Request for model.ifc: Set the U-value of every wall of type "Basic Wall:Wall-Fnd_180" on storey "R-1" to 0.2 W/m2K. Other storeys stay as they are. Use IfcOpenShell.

First a look at what the model holds.

```python
import ifcopenshell
import ifcopenshell.util.element

model = ifcopenshell.open("model.ifc")
print(model.schema)
storey = next(s for s in model.by_type("IfcBuildingStorey") if s.Name == "R-1")
walls = [e for e in ifcopenshell.util.element.get_decomposition(storey) if e.is_a("IfcWall")]
seen = {}
for e in walls:
    element_type = ifcopenshell.util.element.get_type(e)
    key = (element_type.Name if element_type != e and element_type else None, ifcopenshell.util.element.get_pset(e, "Pset_WallCommon", "ThermalTransmittance"))
    seen[key] = seen.get(key, 0) + 1
for (name, value), count in sorted(seen.items(), key=str):
    print(count, "x", name, "|", value)
```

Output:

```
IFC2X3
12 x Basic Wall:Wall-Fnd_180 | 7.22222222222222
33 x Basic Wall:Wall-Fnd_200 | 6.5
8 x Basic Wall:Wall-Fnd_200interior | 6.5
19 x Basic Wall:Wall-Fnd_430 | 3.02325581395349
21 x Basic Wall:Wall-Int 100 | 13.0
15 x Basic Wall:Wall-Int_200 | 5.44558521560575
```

```python
import ifcopenshell
import ifcopenshell.api.pset
import ifcopenshell.util.element

model = ifcopenshell.open("model.ifc")

storey = next(s for s in model.by_type("IfcBuildingStorey") if s.Name == "R-1")
walls = [e for e in ifcopenshell.util.element.get_decomposition(storey) if e.is_a("IfcWall")]

count = 0
for e in walls:
    element_type = ifcopenshell.util.element.get_type(e)
    if element_type in (None, e) or element_type.Name != "Basic Wall:Wall-Fnd_180":
        continue
    # add_pset returns the element's existing set when there is one.
    pset = ifcopenshell.api.pset.add_pset(model, product=e, name="Pset_WallCommon")
    ifcopenshell.api.pset.edit_pset(model, pset=pset, properties={"ThermalTransmittance": 0.2})
    count += 1

print(count, "walls updated")

model.write("model_v2.ifc")
```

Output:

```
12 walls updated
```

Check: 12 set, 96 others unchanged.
